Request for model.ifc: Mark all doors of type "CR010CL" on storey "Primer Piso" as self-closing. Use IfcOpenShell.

First a look at what the model holds.

```python
import ifcopenshell
import ifcopenshell.util.element

model = ifcopenshell.open("model.ifc")
print(model.schema)
storey = next(s for s in model.by_type("IfcBuildingStorey") if s.Name == "Primer Piso")
doors = [e for e in ifcopenshell.util.element.get_decomposition(storey) if e.is_a("IfcDoor")]
seen = {}
for e in doors:
    element_type = ifcopenshell.util.element.get_type(e)
    key = (element_type.Name if element_type != e and element_type else None, ifcopenshell.util.element.get_pset(e, "Pset_DoorCommon", "SelfClosing"))
    seen[key] = seen.get(key, 0) + 1
for (name, value), count in sorted(seen.items(), key=str):
    print(count, "x", name, "|", value)
```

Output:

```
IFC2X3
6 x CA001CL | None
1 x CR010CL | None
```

```python
import ifcopenshell
import ifcopenshell.api.pset
import ifcopenshell.util.element

model = ifcopenshell.open("model.ifc")

storey = next(s for s in model.by_type("IfcBuildingStorey") if s.Name == "Primer Piso")
doors = [e for e in ifcopenshell.util.element.get_decomposition(storey) if e.is_a("IfcDoor")]

count = 0
for e in doors:
    element_type = ifcopenshell.util.element.get_type(e)
    if element_type in (None, e) or element_type.Name != "CR010CL":
        continue
    # add_pset returns the element's existing set when there is one.
    pset = ifcopenshell.api.pset.add_pset(model, product=e, name="Pset_DoorCommon")
    ifcopenshell.api.pset.edit_pset(model, pset=pset, properties={"SelfClosing": True})
    count += 1

print(count, "doors updated")

model.write("model-out.ifc")
```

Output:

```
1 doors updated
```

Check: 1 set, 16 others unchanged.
